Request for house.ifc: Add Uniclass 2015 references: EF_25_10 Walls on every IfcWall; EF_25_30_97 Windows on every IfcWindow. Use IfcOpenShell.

First a look at what the model holds.

```python
import ifcopenshell

model = ifcopenshell.open("house.ifc")
print(model.schema)
print("classifications:", [c.Name for c in model.by_type("IfcClassification")])
for ifc_class in ("IfcDoor", "IfcRoof", "IfcStair", "IfcWall", "IfcWindow"):
    print(ifc_class, len(model.by_type(ifc_class)))
```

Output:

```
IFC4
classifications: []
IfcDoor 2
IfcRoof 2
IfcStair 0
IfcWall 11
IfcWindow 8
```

```python
import ifcopenshell
import ifcopenshell.api.classification

model = ifcopenshell.open("house.ifc")

system = ifcopenshell.api.classification.add_classification(model, classification="Uniclass 2015")

codes = {
    "IfcWall": ("EF_25_10", "Walls"),
    "IfcWindow": ("EF_25_30_97", "Windows"),
}
for ifc_class, (code, name) in codes.items():
    products = model.by_type(ifc_class)
    ifcopenshell.api.classification.add_reference(
        model, products=products, classification=system, identification=code, name=name
    )
    print(code, len(products))

model.write("house_updated.ifc")
```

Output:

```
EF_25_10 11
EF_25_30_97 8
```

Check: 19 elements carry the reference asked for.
